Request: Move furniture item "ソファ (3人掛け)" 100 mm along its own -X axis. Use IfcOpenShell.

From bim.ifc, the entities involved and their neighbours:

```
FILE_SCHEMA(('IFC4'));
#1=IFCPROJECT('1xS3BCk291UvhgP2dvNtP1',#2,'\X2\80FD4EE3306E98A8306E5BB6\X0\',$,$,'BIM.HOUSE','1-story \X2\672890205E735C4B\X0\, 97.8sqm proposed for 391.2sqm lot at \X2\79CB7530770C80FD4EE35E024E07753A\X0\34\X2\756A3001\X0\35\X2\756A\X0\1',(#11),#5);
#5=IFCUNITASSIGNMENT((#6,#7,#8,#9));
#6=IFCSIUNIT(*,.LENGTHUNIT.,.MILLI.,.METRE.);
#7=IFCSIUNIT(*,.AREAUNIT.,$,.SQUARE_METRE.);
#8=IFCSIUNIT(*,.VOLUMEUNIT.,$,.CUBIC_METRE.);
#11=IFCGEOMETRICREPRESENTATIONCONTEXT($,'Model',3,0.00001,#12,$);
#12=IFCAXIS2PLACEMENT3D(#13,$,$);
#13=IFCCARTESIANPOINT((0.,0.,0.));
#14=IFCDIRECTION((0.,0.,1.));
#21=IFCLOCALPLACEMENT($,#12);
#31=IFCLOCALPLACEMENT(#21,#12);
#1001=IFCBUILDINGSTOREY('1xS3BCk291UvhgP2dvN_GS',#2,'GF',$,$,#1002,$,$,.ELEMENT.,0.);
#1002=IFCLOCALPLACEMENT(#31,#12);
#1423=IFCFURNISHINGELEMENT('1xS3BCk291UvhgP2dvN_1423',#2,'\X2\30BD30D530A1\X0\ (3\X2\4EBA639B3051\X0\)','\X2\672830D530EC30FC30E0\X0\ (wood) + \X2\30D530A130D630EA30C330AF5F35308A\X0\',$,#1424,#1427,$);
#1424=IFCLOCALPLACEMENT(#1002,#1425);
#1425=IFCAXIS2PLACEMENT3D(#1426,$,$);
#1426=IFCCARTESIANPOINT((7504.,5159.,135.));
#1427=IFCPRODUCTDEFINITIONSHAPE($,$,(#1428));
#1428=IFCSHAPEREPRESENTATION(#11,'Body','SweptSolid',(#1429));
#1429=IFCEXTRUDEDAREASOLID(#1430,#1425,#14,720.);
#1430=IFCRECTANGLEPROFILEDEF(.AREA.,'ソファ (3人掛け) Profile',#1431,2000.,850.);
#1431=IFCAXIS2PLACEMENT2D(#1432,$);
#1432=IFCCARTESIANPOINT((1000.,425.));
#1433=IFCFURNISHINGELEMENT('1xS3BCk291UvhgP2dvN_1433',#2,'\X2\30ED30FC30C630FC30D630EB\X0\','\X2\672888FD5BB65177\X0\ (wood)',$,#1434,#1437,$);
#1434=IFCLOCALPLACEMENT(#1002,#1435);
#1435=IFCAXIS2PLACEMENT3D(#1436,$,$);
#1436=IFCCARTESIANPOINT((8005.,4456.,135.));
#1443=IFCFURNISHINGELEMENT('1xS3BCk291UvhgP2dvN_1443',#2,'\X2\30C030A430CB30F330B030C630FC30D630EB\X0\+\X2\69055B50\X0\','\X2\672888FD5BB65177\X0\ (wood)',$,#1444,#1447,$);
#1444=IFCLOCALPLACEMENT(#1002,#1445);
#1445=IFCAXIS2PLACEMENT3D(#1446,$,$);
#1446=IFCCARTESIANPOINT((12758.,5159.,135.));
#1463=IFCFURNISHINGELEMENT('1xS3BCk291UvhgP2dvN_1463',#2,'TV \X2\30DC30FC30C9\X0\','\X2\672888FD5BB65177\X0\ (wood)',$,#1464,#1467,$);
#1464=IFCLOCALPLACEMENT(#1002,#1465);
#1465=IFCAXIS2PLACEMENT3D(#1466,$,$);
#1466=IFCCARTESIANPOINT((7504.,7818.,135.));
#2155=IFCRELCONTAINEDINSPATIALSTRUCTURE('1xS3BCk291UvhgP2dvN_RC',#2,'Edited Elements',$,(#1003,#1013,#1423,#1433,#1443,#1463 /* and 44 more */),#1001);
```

```python
import ifcopenshell
import ifcopenshell.api.geometry
import ifcopenshell.util.placement
import ifcopenshell.util.unit

model = ifcopenshell.open("bim.ifc")
unit_scale = ifcopenshell.util.unit.calculate_unit_scale(model)

item = model.by_id(1423)
matrix = ifcopenshell.util.placement.get_local_placement(item.ObjectPlacement)
matrix[:3, 3] -= matrix[:3, 0] * 0.1 / unit_scale
ifcopenshell.api.geometry.edit_object_placement(model, product=item, matrix=matrix, is_si=False)

print(ifcopenshell.util.placement.get_local_placement(item.ObjectPlacement).round(3) + 0.0)

model.write("bim_rev.ifc")
```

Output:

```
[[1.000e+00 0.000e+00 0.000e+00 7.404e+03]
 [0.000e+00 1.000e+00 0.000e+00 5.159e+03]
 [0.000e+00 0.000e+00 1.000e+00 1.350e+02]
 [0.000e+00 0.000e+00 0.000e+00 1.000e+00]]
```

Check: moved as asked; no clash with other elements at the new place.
